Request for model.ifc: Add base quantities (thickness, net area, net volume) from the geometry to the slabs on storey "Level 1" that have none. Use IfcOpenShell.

First a look at what the model holds.

```python
import ifcopenshell
import ifcopenshell.util.element
import ifcopenshell.util.unit

model = ifcopenshell.open("model.ifc")
print(model.schema)
for unit_type in ("LENGTHUNIT", "AREAUNIT", "VOLUMEUNIT"):
    print(unit_type, ifcopenshell.util.unit.calculate_unit_scale(model, unit_type))
storey = next(s for s in model.by_type("IfcBuildingStorey") if s.Name == "Level 1")
slabs = [e for e in ifcopenshell.util.element.get_decomposition(storey) if e.is_a("IfcSlab")]
for e in sorted(slabs, key=lambda e: e.id()):
    print(e.id(), e.is_a(), e.Name, list(ifcopenshell.util.element.get_psets(e, qtos_only=True)), sep=" | ")
```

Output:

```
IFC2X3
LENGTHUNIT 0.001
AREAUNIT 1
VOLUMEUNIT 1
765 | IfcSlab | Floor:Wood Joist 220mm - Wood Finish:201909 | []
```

```python
import ifcopenshell
import ifcopenshell.api.pset
import ifcopenshell.geom
import ifcopenshell.util.element
import ifcopenshell.util.shape
import ifcopenshell.util.unit

model = ifcopenshell.open("model.ifc")
unit_scale = ifcopenshell.util.unit.calculate_unit_scale(model)
area_scale = ifcopenshell.util.unit.calculate_unit_scale(model, "AREAUNIT")
volume_scale = ifcopenshell.util.unit.calculate_unit_scale(model, "VOLUMEUNIT")
settings = ifcopenshell.geom.settings()

storey = next(s for s in model.by_type("IfcBuildingStorey") if s.Name == "Level 1")
slabs = [e for e in ifcopenshell.util.element.get_decomposition(storey) if e.is_a("IfcSlab")]

for e in sorted(slabs, key=lambda e: e.id()):
    if ifcopenshell.util.element.get_psets(e, qtos_only=True, should_inherit=False):
        continue
    # Geometry comes back in metres, in the element's own axes.
    shape = ifcopenshell.geom.create_shape(settings, e)
    values = {
        "Width": ifcopenshell.util.shape.get_z(shape.geometry) / unit_scale,
        "NetArea": ifcopenshell.util.shape.get_footprint_area(shape.geometry) / area_scale,
        "NetVolume": ifcopenshell.util.shape.get_volume(shape.geometry) / volume_scale,
    }
    qto = ifcopenshell.api.pset.add_qto(model, product=e, name="BaseQuantities")
    ifcopenshell.api.pset.edit_qto(model, qto=qto, properties=values)
    print(e.id(), {k: round(v, 3) for k, v in values.items()})

model.write("model_v2.ifc")
```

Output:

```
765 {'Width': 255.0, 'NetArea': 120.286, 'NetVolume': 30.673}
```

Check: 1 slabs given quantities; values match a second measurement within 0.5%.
